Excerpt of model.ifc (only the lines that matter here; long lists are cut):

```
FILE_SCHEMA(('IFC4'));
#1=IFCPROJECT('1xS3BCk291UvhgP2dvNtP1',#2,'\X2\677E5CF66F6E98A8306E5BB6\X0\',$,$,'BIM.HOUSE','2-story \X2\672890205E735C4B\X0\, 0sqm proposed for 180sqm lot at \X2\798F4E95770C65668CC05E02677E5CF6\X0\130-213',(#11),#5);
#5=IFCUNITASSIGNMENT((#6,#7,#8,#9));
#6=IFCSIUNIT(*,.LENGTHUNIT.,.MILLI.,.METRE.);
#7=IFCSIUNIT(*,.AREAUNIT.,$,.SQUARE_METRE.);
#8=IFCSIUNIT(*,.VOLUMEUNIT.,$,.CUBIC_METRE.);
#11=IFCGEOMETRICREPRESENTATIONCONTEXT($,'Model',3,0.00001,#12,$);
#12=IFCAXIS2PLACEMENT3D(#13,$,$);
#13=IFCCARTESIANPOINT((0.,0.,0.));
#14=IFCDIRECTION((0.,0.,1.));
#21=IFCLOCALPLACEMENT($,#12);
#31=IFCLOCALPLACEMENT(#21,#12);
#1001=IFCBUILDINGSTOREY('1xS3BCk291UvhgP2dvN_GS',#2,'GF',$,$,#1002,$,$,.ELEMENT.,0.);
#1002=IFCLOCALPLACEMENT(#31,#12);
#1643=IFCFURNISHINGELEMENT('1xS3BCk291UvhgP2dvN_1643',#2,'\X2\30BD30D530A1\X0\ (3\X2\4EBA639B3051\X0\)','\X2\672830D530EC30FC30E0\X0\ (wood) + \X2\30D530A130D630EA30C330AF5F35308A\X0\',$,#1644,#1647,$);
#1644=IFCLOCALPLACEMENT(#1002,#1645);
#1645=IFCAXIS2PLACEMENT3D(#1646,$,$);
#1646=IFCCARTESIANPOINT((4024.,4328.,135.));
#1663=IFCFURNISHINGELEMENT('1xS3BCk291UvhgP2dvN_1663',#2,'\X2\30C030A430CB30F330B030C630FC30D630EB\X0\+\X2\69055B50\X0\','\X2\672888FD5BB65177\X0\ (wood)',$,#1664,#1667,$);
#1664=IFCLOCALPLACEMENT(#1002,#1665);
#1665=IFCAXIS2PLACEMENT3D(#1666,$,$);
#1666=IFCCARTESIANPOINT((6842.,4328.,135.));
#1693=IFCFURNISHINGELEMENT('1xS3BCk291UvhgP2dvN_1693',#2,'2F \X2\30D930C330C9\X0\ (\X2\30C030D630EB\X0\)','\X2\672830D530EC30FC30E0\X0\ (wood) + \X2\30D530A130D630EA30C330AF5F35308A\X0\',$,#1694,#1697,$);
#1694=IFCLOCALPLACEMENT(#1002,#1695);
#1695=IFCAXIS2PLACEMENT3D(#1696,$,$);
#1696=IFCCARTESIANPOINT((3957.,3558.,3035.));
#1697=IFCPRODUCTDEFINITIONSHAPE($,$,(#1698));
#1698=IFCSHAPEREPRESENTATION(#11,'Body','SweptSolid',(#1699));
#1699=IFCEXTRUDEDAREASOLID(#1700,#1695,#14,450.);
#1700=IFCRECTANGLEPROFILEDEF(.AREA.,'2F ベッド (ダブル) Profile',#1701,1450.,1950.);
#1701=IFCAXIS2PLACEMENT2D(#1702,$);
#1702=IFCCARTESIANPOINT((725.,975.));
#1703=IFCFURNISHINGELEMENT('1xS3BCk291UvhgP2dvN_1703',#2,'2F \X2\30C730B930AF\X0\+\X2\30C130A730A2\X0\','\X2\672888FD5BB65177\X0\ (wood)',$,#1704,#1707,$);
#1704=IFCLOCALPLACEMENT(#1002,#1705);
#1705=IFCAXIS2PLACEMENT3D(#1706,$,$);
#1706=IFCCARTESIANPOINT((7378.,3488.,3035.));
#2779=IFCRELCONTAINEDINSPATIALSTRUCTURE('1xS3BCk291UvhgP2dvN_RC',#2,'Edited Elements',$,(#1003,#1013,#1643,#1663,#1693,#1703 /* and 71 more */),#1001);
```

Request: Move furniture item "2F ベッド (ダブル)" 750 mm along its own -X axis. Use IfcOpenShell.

```python
import ifcopenshell
import ifcopenshell.api.geometry
import ifcopenshell.util.placement

model = ifcopenshell.open("model.ifc")

item = model.by_guid("1xS3BCk291UvhgP2dvN_1693")
matrix = ifcopenshell.util.placement.get_local_placement(item.ObjectPlacement)
matrix[:3, 3] -= matrix[:3, 0] * 750.0
ifcopenshell.api.geometry.edit_object_placement(model, product=item, matrix=matrix, is_si=False)

print(ifcopenshell.util.placement.get_local_placement(item.ObjectPlacement).round(3) + 0.0)

model.write("model_rev.ifc")
```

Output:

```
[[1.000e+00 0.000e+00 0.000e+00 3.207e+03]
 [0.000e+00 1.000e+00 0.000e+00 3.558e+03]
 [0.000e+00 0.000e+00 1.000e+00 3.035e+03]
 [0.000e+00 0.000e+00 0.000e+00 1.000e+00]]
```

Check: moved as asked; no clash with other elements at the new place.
